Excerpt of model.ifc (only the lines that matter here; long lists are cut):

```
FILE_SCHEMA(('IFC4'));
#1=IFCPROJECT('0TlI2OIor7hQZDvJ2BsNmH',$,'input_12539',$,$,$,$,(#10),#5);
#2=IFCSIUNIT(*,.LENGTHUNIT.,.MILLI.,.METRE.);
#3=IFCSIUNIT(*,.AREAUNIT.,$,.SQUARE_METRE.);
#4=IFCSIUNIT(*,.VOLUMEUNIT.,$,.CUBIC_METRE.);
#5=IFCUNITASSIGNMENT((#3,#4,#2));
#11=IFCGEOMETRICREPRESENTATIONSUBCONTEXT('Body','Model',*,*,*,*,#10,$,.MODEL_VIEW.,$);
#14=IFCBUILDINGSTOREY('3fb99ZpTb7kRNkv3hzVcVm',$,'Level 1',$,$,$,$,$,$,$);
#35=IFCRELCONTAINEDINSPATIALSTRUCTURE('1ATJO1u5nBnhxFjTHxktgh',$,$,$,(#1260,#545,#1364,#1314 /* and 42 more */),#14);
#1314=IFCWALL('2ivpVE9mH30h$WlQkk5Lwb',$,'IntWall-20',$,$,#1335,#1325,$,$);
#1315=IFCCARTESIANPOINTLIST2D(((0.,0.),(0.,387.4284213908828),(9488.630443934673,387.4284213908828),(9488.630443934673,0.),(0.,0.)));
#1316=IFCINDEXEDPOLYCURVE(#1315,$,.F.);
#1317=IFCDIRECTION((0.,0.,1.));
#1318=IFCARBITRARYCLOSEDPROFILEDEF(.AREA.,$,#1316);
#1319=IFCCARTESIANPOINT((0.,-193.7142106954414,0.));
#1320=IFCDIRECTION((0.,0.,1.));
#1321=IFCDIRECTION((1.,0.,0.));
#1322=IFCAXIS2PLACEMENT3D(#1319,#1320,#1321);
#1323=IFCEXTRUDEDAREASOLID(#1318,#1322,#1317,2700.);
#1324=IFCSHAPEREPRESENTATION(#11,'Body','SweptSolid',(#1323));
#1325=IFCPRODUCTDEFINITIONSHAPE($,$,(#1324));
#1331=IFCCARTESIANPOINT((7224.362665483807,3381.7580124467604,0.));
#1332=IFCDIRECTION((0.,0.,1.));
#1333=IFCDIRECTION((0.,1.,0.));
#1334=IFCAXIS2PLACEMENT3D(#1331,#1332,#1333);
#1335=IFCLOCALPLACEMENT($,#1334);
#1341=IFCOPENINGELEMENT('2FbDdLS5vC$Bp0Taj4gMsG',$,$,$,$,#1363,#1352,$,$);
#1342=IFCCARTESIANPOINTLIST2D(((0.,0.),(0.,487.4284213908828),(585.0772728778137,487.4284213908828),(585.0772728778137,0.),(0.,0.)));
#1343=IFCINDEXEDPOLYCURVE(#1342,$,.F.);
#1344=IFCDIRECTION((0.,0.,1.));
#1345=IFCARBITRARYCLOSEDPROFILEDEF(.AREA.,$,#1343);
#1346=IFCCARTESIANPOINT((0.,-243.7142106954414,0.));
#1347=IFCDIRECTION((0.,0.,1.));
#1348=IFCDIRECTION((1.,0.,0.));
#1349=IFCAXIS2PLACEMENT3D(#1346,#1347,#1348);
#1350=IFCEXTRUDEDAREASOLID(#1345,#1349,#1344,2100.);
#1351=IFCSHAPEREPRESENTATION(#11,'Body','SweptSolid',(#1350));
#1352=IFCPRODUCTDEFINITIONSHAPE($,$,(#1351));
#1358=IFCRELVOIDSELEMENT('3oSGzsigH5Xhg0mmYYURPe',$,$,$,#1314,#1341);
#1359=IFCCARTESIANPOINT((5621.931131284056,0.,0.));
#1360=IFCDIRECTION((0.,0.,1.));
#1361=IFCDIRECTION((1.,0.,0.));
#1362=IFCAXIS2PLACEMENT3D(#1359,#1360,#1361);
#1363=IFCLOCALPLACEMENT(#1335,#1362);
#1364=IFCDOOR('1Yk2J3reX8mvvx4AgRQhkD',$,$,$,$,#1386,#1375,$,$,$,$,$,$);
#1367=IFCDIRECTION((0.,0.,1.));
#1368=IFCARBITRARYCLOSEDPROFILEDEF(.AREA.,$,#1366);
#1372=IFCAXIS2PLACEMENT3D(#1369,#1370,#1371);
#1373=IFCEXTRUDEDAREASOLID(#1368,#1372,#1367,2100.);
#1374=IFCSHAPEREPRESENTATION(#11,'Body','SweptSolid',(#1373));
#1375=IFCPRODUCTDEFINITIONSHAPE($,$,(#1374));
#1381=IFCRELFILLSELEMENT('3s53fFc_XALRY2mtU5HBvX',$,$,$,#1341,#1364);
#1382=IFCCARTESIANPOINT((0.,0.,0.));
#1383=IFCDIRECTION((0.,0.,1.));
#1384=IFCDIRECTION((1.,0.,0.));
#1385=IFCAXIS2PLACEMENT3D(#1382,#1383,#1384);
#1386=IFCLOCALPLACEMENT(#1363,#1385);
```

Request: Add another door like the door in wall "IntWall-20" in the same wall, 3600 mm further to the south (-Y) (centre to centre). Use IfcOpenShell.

```python
import ifcopenshell
import ifcopenshell.api.feature
import ifcopenshell.api.geometry
import ifcopenshell.api.root
import ifcopenshell.geom
import ifcopenshell.util.element
import ifcopenshell.util.placement
import ifcopenshell.util.shape

model = ifcopenshell.open("model.ifc")
settings = ifcopenshell.geom.settings()


def volume(element):
    """Net volume in cubic metres, openings subtracted."""
    shape = ifcopenshell.geom.create_shape(settings, element)
    return ifcopenshell.util.shape.get_volume(shape.geometry)


door = model.by_id(1364)
opening = door.FillsVoids[0].RelatingOpeningElement
wall = opening.VoidsElements[0].RelatingBuildingElement
before = volume(wall)
shift = ifcopenshell.util.placement.get_local_placement(wall.ObjectPlacement)[:3, 0] * -3600.0

# copy_class copies the void relationship, type, container and properties, but no geometry.
new_opening = ifcopenshell.api.root.copy_class(model, product=opening)
new_opening.Representation = ifcopenshell.util.element.copy_deep(
    model, opening.Representation, exclude=["IfcGeometricRepresentationContext", "IfcRepresentationMap"]
)
new_door = ifcopenshell.api.root.copy_class(model, product=door)
new_door.Representation = ifcopenshell.util.element.copy_deep(
    model, door.Representation, exclude=["IfcGeometricRepresentationContext", "IfcRepresentationMap"]
)
ifcopenshell.api.feature.add_filling(model, opening=new_opening, element=new_door)

for old, new in ((opening, new_opening), (door, new_door)):
    matrix = ifcopenshell.util.placement.get_local_placement(old.ObjectPlacement)
    matrix[:3, 3] += shift
    ifcopenshell.api.geometry.edit_object_placement(model, product=new, matrix=matrix, is_si=False)

after = volume(wall)

print(f"wall volume {before:.3f} -> {after:.3f} m3")

model.write("model_edited.ifc")
```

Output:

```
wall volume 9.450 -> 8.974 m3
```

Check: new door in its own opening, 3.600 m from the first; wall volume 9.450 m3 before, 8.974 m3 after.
